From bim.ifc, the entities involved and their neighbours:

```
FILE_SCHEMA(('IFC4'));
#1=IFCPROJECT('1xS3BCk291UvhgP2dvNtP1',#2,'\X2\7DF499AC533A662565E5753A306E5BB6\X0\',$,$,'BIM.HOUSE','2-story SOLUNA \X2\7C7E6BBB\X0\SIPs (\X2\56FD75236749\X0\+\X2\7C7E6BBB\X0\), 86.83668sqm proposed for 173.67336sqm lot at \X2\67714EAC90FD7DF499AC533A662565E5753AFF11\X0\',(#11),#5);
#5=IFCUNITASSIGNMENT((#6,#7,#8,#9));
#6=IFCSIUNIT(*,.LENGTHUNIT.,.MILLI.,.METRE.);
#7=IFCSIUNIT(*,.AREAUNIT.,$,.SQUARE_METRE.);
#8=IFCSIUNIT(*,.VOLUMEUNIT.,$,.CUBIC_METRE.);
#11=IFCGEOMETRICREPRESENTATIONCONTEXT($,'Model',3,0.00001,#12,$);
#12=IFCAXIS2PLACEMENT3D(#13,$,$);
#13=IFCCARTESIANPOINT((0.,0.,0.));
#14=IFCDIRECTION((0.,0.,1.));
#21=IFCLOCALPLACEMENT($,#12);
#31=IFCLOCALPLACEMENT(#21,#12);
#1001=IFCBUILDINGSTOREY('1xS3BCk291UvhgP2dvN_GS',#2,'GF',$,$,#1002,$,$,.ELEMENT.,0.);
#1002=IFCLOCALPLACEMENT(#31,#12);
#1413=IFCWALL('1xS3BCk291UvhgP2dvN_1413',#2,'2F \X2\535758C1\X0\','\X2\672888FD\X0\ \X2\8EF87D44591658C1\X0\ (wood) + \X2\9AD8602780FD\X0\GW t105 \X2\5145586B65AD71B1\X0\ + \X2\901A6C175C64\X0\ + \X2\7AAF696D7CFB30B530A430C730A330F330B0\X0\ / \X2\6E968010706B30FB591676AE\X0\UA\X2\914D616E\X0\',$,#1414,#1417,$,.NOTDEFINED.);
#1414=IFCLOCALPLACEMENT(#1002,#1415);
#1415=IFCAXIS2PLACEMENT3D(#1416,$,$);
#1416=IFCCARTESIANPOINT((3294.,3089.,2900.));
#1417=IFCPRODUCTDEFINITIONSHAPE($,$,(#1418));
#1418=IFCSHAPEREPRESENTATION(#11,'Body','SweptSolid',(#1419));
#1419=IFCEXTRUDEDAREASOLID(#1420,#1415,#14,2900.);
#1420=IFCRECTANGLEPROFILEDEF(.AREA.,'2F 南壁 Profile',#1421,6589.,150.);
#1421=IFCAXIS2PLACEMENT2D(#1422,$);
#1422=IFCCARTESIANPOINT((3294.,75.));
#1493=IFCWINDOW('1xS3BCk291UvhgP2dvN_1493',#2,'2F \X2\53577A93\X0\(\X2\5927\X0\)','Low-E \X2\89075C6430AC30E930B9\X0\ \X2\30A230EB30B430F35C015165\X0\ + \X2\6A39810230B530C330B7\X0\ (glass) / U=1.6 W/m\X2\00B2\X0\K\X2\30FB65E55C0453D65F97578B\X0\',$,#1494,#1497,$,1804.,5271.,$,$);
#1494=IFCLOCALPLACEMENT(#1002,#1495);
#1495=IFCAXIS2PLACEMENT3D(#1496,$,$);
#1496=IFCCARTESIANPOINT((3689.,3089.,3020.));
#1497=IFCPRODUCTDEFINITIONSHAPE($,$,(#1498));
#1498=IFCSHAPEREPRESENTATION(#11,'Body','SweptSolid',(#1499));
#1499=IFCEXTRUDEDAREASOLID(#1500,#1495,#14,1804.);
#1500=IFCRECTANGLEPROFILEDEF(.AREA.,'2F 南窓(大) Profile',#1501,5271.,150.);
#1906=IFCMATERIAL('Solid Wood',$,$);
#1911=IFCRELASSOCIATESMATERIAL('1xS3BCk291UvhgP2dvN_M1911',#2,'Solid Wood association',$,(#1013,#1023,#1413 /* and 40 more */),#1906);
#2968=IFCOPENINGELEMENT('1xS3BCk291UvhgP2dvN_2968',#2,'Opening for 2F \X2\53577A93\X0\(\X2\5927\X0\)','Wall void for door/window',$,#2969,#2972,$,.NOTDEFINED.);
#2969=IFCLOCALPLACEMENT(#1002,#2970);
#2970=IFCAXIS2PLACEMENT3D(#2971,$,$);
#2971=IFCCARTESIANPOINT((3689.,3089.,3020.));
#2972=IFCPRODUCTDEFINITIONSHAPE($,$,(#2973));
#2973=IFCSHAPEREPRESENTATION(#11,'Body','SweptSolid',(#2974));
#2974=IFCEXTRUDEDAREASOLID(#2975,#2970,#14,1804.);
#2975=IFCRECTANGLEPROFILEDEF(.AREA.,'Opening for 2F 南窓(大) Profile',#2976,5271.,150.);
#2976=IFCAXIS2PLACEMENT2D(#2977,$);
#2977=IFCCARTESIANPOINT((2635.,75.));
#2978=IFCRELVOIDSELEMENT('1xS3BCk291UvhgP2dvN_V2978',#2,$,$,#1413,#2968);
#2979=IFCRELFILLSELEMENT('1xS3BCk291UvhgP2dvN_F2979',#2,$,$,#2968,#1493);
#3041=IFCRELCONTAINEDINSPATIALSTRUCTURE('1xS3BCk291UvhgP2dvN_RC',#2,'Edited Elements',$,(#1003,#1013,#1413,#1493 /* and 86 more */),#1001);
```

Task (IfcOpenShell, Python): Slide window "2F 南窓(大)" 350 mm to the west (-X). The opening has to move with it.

```python
import ifcopenshell
import ifcopenshell.api.geometry
import ifcopenshell.util.placement

model = ifcopenshell.open("bim.ifc")

window = model.by_guid("1xS3BCk291UvhgP2dvN_1493")
opening = window.FillsVoids[0].RelatingOpeningElement
wall = opening.VoidsElements[0].RelatingBuildingElement

wall_matrix = ifcopenshell.util.placement.get_local_placement(wall.ObjectPlacement)
shift = wall_matrix[:3, 0] * -350.0
before = ifcopenshell.util.placement.get_local_placement(window.ObjectPlacement)[:3, 3].copy()

# The window is not placed relative to its opening, so move both.
for product in (opening, window):
    matrix = ifcopenshell.util.placement.get_local_placement(product.ObjectPlacement)
    matrix[:3, 3] += shift
    ifcopenshell.api.geometry.edit_object_placement(model, product=product, matrix=matrix, is_si=False)

after = ifcopenshell.util.placement.get_local_placement(window.ObjectPlacement)[:3, 3]
print("window moved by", (after - before).round(3) + 0.0)

model.write("bim-out.ifc")
```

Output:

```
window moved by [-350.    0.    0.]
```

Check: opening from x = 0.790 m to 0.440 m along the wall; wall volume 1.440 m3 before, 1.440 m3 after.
